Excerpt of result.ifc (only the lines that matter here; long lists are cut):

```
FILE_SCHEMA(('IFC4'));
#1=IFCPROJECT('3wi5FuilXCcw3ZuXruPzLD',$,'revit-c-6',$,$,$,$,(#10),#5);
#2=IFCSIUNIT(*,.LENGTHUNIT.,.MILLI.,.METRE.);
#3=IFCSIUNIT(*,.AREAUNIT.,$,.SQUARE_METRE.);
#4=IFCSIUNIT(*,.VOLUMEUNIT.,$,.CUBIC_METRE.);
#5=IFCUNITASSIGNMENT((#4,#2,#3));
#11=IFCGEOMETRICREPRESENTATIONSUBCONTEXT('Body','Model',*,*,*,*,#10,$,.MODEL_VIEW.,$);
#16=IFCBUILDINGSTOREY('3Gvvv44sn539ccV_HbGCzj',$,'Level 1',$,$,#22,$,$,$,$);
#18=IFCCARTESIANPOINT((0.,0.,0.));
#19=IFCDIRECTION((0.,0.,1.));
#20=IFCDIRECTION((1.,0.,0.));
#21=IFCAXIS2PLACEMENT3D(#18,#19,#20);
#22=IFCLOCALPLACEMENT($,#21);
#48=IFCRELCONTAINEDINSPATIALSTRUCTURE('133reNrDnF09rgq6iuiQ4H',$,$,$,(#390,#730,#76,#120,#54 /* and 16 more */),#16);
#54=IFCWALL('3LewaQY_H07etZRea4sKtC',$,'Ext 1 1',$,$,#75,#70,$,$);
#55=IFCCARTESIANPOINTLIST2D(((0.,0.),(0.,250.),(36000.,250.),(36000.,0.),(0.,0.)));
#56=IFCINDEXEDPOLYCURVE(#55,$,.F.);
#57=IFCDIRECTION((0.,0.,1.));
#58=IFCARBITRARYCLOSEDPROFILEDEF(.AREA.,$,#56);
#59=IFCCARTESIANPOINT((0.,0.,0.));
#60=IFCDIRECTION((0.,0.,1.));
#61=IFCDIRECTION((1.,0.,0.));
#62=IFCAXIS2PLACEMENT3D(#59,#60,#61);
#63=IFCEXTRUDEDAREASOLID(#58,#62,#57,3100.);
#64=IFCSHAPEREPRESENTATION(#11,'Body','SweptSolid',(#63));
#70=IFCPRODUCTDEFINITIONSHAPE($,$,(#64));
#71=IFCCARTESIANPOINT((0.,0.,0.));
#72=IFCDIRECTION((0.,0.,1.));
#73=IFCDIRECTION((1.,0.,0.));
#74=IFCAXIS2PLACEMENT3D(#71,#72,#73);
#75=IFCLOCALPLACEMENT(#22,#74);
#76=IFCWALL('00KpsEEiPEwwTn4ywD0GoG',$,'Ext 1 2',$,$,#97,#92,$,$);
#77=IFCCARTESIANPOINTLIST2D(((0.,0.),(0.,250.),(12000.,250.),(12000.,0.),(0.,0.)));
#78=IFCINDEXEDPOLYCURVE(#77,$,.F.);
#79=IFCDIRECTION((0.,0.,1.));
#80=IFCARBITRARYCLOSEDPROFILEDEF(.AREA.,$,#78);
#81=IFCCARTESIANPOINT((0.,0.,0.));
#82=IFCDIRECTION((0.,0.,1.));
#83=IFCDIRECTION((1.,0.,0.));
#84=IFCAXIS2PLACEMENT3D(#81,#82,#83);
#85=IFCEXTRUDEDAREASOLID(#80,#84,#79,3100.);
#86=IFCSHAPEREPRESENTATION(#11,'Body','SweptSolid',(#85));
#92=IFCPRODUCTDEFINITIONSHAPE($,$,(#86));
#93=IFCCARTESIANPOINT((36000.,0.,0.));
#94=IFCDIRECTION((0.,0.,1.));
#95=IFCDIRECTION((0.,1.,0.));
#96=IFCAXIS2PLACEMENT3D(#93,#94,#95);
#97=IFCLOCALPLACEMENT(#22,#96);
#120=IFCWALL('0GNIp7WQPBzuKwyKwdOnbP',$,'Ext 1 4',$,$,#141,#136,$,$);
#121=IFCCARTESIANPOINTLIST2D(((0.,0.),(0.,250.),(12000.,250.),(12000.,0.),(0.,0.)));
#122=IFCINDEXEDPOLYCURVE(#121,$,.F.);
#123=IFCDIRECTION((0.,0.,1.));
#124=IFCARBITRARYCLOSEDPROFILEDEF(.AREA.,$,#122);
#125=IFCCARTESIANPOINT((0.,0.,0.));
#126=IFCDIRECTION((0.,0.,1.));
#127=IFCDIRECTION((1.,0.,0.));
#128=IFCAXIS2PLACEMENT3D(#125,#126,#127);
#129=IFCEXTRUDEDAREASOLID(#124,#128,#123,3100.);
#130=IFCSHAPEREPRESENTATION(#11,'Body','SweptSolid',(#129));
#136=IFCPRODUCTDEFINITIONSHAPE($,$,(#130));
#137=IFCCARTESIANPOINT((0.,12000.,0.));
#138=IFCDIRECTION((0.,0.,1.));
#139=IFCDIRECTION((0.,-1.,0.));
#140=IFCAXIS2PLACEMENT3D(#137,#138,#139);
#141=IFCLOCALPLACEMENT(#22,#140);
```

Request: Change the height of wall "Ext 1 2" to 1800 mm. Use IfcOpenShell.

```python
import ifcopenshell
import ifcopenshell.geom
import ifcopenshell.util.representation
import ifcopenshell.util.shape
import ifcopenshell.util.unit

model = ifcopenshell.open("result.ifc")
unit_scale = ifcopenshell.util.unit.calculate_unit_scale(model)
settings = ifcopenshell.geom.settings()


def volume(element):
    """Net volume in cubic metres, openings subtracted."""
    shape = ifcopenshell.geom.create_shape(settings, element)
    return ifcopenshell.util.shape.get_volume(shape.geometry)


wall = model.by_id(76)
before = volume(wall)

body = ifcopenshell.util.representation.get_representation(wall, "Model", "Body")
solid = body.Items[0]
old_height = solid.Depth
solid.Depth = 1.8 / unit_scale
after = volume(wall)

print(f"height {old_height:g} -> {solid.Depth:g}, volume {before:.3f} -> {after:.3f} m3")

model.write("result_v2.ifc")
```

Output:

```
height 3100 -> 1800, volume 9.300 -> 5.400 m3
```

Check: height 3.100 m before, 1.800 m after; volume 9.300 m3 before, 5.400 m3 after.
